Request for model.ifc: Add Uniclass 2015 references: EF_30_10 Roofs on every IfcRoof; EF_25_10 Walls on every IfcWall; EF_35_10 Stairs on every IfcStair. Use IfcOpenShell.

First a look at what the model holds.

```python
import ifcopenshell

model = ifcopenshell.open("model.ifc")
print(model.schema)
print("classifications:", [c.Name for c in model.by_type("IfcClassification")])
for ifc_class in ("IfcDoor", "IfcRoof", "IfcStair", "IfcWall", "IfcWindow"):
    print(ifc_class, len(model.by_type(ifc_class)))
```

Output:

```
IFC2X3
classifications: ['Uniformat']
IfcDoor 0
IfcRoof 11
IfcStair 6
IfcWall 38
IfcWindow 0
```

```python
import ifcopenshell
import ifcopenshell.api.classification

model = ifcopenshell.open("model.ifc")

# IFC2X3 requires Source and Edition and has no link from the project to the system.
system = model.create_entity("IfcClassification", Source="NBS", Edition="2015", Name="Uniclass 2015")

codes = {
    "IfcRoof": ("EF_30_10", "Roofs"),
    "IfcWall": ("EF_25_10", "Walls"),
    "IfcStair": ("EF_35_10", "Stairs"),
}
for ifc_class, (code, name) in codes.items():
    products = model.by_type(ifc_class)
    ifcopenshell.api.classification.add_reference(
        model, products=products, classification=system, identification=code, name=name
    )
    print(code, len(products))

model.write("model_updated.ifc")
```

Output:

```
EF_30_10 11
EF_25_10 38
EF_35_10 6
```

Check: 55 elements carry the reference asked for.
